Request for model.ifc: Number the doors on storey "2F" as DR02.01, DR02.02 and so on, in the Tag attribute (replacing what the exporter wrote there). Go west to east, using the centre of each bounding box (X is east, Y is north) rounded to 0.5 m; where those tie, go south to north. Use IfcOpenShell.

First a look at what the model holds.

```python
import ifcopenshell
import ifcopenshell.util.element
import ifcopenshell.util.placement

model = ifcopenshell.open("model.ifc")
print(model.schema)
storey = next(s for s in model.by_type("IfcBuildingStorey") if s.Name == "2F")
doors = [e for e in ifcopenshell.util.element.get_decomposition(storey) if e.is_a("IfcDoor")]
for e in sorted(doors, key=lambda e: e.id()):
    origin = ifcopenshell.util.placement.get_local_placement(e.ObjectPlacement)[:3, 3]
    print(e.id(), e.Tag, e.Name, origin.round(2) + 0.0, sep=" | ")
```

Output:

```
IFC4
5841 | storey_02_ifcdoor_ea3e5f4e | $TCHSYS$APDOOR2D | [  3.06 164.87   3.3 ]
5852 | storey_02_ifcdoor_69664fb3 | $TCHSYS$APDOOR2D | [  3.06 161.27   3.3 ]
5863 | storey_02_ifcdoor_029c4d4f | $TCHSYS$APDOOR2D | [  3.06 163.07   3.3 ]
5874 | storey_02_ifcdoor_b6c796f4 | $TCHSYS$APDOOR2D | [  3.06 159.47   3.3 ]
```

```python
import ifcopenshell
import ifcopenshell.geom
import ifcopenshell.util.element
import ifcopenshell.util.shape

model = ifcopenshell.open("model.ifc")
settings = ifcopenshell.geom.settings()
settings.set("use-world-coords", True)


def centre(element):
    shape = ifcopenshell.geom.create_shape(settings, element)
    return ifcopenshell.util.shape.get_bbox_centroid(shape.geometry)


storey = next(s for s in model.by_type("IfcBuildingStorey") if s.Name == "2F")
doors = [e for e in ifcopenshell.util.element.get_decomposition(storey) if e.is_a("IfcDoor")]

# Insertion points can sit at a corner or the storey origin, so sort by the geometry (in metres).
centres = {e: centre(e) for e in doors}
doors.sort(key=lambda e: (round(centres[e][0] / 0.5), centres[e][1]))

for i, e in enumerate(doors, start=1):
    number = f"DR02.{i:02d}"
    e.Tag = number
    print(e.id(), number)

model.write("model_edited.ifc")
```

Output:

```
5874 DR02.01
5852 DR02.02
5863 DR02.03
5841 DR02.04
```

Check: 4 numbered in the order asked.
